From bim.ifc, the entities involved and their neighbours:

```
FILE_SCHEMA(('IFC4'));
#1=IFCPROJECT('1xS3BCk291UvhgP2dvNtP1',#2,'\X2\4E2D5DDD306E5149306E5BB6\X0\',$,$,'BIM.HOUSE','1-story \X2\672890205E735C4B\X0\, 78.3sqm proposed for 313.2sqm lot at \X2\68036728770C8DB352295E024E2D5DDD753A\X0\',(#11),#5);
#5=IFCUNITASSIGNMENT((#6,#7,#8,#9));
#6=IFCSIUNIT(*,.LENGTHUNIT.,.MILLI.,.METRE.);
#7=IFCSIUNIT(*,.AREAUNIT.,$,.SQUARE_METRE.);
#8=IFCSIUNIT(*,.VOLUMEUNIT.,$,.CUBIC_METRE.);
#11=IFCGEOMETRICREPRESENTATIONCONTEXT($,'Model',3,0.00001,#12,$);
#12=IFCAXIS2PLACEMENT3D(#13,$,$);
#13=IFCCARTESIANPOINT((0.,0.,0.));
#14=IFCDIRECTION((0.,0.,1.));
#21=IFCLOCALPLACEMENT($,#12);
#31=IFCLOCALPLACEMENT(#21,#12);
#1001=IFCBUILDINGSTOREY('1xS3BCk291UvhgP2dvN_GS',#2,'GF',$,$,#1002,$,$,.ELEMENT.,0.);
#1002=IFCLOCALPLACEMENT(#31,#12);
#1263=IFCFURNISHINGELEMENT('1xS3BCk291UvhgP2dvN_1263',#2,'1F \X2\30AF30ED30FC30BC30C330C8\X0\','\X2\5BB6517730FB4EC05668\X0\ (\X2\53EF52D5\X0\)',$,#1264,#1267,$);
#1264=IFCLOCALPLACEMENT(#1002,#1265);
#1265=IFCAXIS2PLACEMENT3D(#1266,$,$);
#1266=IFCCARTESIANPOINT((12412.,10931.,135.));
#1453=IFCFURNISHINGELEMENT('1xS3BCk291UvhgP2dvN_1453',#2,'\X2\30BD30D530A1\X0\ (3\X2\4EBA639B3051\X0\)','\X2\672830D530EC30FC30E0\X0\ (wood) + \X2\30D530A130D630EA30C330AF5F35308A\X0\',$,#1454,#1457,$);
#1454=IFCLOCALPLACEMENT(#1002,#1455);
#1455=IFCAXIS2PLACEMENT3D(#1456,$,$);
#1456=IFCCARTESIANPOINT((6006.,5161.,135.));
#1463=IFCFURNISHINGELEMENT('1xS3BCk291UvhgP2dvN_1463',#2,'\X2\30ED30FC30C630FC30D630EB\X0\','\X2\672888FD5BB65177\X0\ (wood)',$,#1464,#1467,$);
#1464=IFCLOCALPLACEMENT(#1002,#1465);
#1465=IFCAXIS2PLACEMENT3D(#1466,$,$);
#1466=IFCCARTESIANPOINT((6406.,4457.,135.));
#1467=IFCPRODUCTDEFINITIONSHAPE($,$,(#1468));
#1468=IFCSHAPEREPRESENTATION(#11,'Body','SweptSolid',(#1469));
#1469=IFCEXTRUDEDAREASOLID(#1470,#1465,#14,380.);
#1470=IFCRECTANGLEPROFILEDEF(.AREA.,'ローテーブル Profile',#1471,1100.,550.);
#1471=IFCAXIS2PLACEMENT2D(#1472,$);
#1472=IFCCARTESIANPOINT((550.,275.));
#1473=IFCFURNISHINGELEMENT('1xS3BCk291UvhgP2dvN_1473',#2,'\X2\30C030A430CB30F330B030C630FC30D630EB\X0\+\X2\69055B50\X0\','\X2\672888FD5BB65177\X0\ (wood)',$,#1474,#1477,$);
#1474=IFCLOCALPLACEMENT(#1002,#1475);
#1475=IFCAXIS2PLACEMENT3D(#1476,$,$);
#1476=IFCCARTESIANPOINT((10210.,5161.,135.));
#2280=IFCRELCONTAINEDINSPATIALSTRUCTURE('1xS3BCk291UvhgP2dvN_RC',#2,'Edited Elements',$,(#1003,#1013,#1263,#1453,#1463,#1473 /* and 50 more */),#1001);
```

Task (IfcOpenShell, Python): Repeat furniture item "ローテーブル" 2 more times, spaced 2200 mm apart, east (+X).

```python
import numpy as np
import ifcopenshell
import ifcopenshell.api.geometry
import ifcopenshell.api.root
import ifcopenshell.util.element
import ifcopenshell.util.placement

model = ifcopenshell.open("bim.ifc")


def reuse_history(source, copy):
    """copy_class also copies each property set's owner history, people and application; keep the originals."""
    for rel in copy.IsDefinedBy:
        if rel.is_a("IfcRelDefinesByProperties") and (history := rel.RelatingPropertyDefinition.OwnerHistory):
            rel.RelatingPropertyDefinition.OwnerHistory = source.OwnerHistory
            ifcopenshell.util.element.remove_deep2(model, history)


source = model.by_guid("1xS3BCk291UvhgP2dvN_1463")
base = ifcopenshell.util.placement.get_local_placement(source.ObjectPlacement)
step = np.array([1.0, 0.0, 0.0]) * 2200.0

for i in range(1, 3):
    copy = ifcopenshell.api.root.copy_class(model, product=source)
    copy.Representation = ifcopenshell.util.element.copy_deep(
        model, source.Representation, exclude=["IfcGeometricRepresentationContext", "IfcRepresentationMap"]
    )
    reuse_history(source, copy)
    matrix = base.copy()
    matrix[:3, 3] += i * step
    print("added at", matrix[:3, 3].round(3) + 0.0)
    ifcopenshell.api.geometry.edit_object_placement(model, product=copy, matrix=matrix, is_si=False)

model.write("bim_edited.ifc")
```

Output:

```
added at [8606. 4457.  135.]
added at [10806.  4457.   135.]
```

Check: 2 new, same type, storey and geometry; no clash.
